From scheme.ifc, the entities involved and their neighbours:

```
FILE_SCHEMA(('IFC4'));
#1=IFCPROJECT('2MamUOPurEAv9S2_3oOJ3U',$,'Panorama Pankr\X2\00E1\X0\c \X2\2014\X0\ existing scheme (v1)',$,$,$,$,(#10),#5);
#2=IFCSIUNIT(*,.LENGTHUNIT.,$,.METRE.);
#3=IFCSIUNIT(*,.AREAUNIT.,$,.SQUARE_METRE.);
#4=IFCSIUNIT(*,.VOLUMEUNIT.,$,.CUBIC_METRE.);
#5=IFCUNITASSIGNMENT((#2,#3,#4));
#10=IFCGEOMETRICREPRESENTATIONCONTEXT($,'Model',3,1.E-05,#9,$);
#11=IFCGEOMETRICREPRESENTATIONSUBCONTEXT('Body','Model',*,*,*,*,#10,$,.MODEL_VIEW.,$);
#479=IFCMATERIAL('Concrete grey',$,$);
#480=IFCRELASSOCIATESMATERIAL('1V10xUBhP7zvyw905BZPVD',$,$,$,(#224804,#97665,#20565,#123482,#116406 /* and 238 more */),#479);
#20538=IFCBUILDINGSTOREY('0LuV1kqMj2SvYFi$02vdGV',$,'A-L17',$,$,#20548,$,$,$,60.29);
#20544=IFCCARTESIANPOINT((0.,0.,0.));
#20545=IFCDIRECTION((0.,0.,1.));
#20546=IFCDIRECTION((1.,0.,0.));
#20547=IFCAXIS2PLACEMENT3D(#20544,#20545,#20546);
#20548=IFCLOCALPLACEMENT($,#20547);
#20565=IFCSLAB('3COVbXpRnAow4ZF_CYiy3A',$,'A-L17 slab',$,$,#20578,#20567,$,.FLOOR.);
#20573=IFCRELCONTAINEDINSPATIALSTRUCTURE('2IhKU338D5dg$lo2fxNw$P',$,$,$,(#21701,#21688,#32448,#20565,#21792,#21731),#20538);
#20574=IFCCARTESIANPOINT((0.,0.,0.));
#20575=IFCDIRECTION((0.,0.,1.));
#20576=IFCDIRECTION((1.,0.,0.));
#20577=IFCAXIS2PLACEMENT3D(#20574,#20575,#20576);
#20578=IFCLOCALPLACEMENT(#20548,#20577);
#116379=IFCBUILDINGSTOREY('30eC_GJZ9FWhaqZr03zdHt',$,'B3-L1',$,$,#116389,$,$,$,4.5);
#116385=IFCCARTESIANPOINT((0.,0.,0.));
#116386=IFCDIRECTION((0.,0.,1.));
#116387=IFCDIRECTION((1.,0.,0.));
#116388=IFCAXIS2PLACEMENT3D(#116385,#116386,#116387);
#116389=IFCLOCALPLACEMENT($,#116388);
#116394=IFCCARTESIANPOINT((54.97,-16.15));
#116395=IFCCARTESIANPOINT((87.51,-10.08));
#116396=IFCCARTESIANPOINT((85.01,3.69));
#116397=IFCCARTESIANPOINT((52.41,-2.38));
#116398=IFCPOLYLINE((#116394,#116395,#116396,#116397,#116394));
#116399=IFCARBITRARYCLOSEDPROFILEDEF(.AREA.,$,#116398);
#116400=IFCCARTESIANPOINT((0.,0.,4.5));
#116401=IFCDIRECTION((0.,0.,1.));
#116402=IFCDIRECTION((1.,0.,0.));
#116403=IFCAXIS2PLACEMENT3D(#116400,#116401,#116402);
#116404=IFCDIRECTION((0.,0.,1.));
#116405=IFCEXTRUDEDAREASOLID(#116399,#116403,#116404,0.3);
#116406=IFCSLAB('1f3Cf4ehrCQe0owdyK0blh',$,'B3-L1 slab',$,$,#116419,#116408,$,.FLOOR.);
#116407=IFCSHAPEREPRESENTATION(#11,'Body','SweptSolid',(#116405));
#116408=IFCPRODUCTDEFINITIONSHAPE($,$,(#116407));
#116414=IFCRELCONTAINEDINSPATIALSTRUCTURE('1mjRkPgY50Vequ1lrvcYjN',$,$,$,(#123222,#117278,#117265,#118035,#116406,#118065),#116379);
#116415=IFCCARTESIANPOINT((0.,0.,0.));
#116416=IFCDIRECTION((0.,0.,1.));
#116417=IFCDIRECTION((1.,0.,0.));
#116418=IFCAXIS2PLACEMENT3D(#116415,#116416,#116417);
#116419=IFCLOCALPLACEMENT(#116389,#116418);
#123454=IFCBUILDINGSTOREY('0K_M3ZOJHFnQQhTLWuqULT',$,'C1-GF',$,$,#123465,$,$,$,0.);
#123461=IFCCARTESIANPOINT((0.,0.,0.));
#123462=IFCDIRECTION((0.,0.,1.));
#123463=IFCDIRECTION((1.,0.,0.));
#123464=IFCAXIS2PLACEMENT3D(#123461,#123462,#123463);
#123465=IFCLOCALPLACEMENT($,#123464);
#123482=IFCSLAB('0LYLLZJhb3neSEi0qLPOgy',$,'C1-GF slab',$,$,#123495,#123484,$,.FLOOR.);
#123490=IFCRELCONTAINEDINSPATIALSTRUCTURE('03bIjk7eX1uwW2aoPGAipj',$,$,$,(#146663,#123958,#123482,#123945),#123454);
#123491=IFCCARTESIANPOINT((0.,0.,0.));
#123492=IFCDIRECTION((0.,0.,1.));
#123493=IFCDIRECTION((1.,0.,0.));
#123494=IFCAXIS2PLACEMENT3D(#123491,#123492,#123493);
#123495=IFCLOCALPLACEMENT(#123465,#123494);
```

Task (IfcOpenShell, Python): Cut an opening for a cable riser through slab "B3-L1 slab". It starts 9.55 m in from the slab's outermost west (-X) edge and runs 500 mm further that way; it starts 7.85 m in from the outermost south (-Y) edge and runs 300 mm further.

```python
import numpy as np
import ifcopenshell
import ifcopenshell.api.feature
import ifcopenshell.api.geometry
import ifcopenshell.api.root
import ifcopenshell.geom
import ifcopenshell.util.placement
import ifcopenshell.util.representation
import ifcopenshell.util.shape
import ifcopenshell.util.unit

model = ifcopenshell.open("scheme.ifc")
unit_scale = ifcopenshell.util.unit.calculate_unit_scale(model)
settings = ifcopenshell.geom.settings()


def volume(element):
    """Net volume in cubic metres, openings subtracted."""
    shape = ifcopenshell.geom.create_shape(settings, element)
    return ifcopenshell.util.shape.get_volume(shape.geometry)


slab = model.by_guid("1f3Cf4ehrCQe0owdyK0blh")
before = volume(slab)

# Extent in the slab's own axes, in metres. The edges named are its -X and -Y sides.
slab_shape = ifcopenshell.geom.create_shape(settings, slab)
vertices = ifcopenshell.util.shape.get_vertices(slab_shape.geometry)
x_min, y_min, bottom = vertices.min(axis=0)
top = vertices[:, 2].max()

opening = ifcopenshell.api.root.create_entity(model, ifc_class="IfcOpeningElement", name="Cable riser opening", predefined_type="OPENING")
context = ifcopenshell.util.representation.get_context(model, "Model", "Body", "MODEL_VIEW")
width, depth = 0.5, 0.3
outline = [(0.0, 0.0), (width, 0.0), (width, depth), (0.0, depth), (0.0, 0.0)]
# Overshoot both faces by 50 mm so the cut is clean.
shape = ifcopenshell.api.geometry.add_slab_representation(
    model, context=context, depth=top - bottom + 0.1, polyline=outline
)
ifcopenshell.api.geometry.assign_representation(model, product=opening, representation=shape)

matrix = ifcopenshell.util.placement.get_local_placement(slab.ObjectPlacement)
matrix[:, 3] = matrix @ np.append(np.array([x_min + 9.55, y_min + 7.85, bottom - 0.05]) / unit_scale, 1.0)
ifcopenshell.api.geometry.edit_object_placement(model, product=opening, matrix=matrix, is_si=False)
ifcopenshell.api.feature.add_feature(model, feature=opening, element=slab)

after = volume(slab)

print(f"slab volume {before:.3f} -> {after:.3f} m3")

model.write("scheme_edited.ifc")
```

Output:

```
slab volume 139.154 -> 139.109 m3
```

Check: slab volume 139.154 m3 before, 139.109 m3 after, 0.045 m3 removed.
